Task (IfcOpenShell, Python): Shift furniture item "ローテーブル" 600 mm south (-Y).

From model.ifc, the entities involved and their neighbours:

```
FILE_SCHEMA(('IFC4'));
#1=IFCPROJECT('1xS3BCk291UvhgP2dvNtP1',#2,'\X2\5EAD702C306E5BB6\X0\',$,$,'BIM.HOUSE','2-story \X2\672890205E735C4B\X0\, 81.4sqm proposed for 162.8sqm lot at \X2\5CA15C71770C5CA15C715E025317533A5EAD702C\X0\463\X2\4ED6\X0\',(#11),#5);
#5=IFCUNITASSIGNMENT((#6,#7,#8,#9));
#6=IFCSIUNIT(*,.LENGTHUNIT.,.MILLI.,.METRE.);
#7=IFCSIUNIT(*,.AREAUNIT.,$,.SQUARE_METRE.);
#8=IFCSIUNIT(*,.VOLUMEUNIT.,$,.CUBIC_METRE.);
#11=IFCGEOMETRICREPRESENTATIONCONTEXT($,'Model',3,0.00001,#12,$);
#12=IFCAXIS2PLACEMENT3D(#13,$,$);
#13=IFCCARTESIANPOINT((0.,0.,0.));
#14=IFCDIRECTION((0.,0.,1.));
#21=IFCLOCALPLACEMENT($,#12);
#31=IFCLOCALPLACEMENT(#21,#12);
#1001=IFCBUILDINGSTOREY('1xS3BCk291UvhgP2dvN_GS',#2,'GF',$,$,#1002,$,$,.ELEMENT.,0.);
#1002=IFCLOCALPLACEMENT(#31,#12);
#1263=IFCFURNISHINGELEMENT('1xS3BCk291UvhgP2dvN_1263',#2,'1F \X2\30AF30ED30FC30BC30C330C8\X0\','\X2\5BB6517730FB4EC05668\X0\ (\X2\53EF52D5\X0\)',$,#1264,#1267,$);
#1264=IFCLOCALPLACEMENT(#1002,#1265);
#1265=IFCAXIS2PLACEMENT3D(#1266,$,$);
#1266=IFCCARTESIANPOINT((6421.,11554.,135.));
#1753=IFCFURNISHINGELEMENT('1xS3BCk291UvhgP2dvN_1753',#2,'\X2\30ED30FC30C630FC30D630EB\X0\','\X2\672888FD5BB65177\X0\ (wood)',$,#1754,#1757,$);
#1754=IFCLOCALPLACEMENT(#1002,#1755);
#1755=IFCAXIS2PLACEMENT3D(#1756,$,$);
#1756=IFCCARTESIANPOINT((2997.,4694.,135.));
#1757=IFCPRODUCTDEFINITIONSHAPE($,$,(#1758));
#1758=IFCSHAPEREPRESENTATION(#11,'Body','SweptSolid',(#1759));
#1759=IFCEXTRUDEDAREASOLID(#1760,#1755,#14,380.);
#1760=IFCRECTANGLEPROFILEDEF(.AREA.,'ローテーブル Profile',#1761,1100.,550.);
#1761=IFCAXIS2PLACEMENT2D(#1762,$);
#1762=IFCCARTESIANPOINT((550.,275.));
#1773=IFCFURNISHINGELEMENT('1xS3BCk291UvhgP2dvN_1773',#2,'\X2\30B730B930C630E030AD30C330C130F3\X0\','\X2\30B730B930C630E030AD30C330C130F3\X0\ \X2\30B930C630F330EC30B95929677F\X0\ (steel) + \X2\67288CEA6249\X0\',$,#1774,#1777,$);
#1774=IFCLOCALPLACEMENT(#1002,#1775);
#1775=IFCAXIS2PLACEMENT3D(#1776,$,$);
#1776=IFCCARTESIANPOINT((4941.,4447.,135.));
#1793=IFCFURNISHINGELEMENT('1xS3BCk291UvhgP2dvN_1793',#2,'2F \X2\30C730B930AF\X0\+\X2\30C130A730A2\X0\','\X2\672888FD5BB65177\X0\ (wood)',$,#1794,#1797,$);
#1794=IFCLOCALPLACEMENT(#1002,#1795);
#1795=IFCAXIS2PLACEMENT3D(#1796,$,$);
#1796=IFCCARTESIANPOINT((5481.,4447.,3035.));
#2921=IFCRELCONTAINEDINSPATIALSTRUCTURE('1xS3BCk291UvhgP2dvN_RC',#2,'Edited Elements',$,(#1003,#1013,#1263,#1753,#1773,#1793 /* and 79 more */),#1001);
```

```python
import ifcopenshell
import ifcopenshell.api.geometry
import ifcopenshell.util.placement
import ifcopenshell.util.unit

model = ifcopenshell.open("model.ifc")
unit_scale = ifcopenshell.util.unit.calculate_unit_scale(model)

item = model.by_guid("1xS3BCk291UvhgP2dvN_1753")
matrix = ifcopenshell.util.placement.get_local_placement(item.ObjectPlacement)
matrix[1, 3] -= 0.6 / unit_scale
ifcopenshell.api.geometry.edit_object_placement(model, product=item, matrix=matrix, is_si=False)

print(ifcopenshell.util.placement.get_local_placement(item.ObjectPlacement).round(3) + 0.0)

model.write("model_v2.ifc")
```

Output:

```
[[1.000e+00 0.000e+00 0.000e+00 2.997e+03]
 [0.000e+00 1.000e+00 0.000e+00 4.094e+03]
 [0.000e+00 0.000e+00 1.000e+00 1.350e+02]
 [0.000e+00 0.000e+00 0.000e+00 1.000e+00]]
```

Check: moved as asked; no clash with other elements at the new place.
